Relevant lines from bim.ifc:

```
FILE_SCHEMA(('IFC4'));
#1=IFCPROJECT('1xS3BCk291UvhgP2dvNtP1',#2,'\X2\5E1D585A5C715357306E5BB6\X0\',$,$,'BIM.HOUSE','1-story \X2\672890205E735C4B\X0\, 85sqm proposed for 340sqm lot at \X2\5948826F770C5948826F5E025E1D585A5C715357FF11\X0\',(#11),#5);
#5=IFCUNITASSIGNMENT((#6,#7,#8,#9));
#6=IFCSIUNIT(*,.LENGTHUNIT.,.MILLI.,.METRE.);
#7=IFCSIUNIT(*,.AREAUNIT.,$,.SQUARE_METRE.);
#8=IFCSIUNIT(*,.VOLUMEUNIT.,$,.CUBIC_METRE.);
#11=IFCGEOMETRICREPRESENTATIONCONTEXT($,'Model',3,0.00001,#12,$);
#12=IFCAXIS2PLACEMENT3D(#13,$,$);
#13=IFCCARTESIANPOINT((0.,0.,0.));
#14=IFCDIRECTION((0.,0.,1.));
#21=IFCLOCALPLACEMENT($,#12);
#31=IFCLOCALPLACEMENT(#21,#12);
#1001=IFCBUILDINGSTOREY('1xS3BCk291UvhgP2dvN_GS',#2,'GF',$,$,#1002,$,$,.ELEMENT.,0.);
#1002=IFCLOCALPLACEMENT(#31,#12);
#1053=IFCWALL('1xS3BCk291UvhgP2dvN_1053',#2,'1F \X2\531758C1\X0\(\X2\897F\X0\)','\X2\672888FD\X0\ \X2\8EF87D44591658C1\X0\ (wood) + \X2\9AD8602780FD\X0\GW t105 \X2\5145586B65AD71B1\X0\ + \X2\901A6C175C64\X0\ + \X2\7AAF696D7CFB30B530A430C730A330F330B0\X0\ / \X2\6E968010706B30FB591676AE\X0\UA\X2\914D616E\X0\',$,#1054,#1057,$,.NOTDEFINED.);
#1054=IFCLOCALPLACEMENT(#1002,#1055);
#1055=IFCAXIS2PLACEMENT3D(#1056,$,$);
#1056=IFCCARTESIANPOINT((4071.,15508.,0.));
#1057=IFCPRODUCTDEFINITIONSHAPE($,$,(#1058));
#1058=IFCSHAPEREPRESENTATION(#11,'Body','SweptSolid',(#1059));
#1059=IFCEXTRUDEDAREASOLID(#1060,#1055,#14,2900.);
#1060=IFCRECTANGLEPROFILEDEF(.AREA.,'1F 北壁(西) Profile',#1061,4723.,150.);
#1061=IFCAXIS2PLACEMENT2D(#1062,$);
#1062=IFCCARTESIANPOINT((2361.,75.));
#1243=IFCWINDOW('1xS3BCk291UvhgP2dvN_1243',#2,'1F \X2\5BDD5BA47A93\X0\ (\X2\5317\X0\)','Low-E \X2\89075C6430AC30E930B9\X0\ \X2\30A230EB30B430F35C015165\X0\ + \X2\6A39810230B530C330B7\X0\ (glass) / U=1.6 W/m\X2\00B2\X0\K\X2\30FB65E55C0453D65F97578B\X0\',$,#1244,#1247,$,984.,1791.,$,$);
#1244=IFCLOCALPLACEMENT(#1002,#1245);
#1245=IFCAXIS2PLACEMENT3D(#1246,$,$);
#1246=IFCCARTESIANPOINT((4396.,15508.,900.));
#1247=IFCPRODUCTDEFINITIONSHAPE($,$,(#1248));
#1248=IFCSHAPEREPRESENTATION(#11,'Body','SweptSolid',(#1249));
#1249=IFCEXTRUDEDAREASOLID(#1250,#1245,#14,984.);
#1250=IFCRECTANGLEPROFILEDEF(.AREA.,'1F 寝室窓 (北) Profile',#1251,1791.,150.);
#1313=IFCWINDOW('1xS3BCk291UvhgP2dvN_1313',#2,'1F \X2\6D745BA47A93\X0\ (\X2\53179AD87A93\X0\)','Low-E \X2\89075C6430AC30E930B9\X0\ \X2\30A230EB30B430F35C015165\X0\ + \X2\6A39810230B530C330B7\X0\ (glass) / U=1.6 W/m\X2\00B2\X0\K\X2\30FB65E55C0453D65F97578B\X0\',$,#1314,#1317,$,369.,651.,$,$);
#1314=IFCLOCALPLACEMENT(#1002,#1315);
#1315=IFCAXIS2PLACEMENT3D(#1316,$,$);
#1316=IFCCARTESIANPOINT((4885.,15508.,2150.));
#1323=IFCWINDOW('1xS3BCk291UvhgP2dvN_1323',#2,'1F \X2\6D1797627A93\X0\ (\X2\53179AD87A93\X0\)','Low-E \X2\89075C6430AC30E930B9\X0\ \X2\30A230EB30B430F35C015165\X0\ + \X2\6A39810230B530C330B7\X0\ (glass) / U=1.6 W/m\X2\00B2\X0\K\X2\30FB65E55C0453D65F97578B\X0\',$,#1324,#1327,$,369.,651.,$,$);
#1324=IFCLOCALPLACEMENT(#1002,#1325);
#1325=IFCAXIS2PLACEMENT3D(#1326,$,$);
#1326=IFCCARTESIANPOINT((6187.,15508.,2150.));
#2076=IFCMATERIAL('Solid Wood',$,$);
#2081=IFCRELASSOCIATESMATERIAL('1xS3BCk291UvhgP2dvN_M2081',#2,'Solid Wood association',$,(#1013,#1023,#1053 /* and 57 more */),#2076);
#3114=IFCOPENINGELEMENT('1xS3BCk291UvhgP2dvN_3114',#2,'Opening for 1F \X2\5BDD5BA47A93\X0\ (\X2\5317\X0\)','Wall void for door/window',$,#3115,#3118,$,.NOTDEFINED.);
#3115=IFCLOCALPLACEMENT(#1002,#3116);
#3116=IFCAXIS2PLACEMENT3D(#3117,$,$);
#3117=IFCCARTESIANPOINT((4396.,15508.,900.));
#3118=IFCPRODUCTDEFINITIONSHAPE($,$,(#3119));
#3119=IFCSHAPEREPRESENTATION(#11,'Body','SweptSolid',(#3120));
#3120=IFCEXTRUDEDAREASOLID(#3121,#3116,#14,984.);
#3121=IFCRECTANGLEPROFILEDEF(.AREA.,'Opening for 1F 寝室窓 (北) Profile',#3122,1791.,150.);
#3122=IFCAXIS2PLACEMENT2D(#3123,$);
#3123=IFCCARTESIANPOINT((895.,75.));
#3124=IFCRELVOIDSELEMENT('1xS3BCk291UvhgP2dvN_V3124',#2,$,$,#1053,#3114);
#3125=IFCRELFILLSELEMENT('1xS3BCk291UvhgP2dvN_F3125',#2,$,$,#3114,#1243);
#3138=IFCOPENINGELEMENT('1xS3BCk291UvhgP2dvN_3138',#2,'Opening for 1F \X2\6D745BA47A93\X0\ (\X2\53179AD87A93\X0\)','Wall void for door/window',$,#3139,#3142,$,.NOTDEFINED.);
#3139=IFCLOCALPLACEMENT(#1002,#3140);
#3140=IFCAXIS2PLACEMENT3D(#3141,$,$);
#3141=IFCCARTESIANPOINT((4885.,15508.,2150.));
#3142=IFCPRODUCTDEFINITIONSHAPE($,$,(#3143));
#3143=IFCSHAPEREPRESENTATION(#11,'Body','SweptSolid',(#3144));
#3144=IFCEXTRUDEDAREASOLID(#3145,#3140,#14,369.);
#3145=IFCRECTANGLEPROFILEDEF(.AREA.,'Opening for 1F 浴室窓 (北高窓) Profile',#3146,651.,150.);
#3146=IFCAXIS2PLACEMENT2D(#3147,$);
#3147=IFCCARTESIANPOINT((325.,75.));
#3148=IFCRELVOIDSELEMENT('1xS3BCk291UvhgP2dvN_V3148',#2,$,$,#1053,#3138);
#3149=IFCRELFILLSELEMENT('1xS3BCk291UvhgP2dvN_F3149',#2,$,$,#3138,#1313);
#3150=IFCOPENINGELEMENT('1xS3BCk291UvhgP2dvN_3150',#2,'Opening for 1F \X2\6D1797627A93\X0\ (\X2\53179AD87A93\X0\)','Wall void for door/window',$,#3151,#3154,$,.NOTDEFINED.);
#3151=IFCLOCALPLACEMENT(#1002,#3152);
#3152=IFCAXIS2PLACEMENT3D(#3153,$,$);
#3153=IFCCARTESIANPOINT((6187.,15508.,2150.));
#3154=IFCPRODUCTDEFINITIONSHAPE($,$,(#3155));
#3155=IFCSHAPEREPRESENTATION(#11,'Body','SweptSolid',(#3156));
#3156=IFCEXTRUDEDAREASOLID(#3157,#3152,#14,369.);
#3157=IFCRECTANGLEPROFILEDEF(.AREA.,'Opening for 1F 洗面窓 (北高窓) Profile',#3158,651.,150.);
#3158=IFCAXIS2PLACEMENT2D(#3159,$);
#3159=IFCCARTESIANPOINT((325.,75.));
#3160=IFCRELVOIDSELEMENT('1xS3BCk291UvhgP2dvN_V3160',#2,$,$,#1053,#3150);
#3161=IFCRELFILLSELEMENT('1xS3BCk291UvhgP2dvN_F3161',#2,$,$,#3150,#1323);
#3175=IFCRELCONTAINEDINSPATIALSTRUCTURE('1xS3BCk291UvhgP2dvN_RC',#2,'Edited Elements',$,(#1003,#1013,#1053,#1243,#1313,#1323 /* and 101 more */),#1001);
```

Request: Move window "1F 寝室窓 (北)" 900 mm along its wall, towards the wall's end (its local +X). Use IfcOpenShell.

```python
import ifcopenshell
import ifcopenshell.api.geometry
import ifcopenshell.util.placement
import ifcopenshell.util.unit

model = ifcopenshell.open("bim.ifc")
unit_scale = ifcopenshell.util.unit.calculate_unit_scale(model)

window = model.by_guid("1xS3BCk291UvhgP2dvN_1243")
opening = window.FillsVoids[0].RelatingOpeningElement
wall = opening.VoidsElements[0].RelatingBuildingElement

wall_matrix = ifcopenshell.util.placement.get_local_placement(wall.ObjectPlacement)
shift = wall_matrix[:3, 0] * 0.9 / unit_scale
before = ifcopenshell.util.placement.get_local_placement(window.ObjectPlacement)[:3, 3].copy()

# The window is not placed relative to its opening, so move both.
for product in (opening, window):
    matrix = ifcopenshell.util.placement.get_local_placement(product.ObjectPlacement)
    matrix[:3, 3] += shift
    ifcopenshell.api.geometry.edit_object_placement(model, product=product, matrix=matrix, is_si=False)

after = ifcopenshell.util.placement.get_local_placement(window.ObjectPlacement)[:3, 3]
print("window moved by", (after - before).round(3) + 0.0)

model.write("bim_updated.ifc")
```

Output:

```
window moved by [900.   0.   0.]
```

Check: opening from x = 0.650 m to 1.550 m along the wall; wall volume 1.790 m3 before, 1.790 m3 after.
